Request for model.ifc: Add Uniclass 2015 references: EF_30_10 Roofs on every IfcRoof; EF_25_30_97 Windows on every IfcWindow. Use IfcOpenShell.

First a look at what the model holds.

```python
import ifcopenshell

model = ifcopenshell.open("model.ifc")
print(model.schema)
print("classifications:", [c.Name for c in model.by_type("IfcClassification")])
for ifc_class in ("IfcDoor", "IfcRoof", "IfcStair", "IfcWall", "IfcWindow"):
    print(ifc_class, len(model.by_type(ifc_class)))
```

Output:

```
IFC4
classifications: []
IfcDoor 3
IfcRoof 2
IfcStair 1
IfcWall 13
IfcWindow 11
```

```python
import ifcopenshell
import ifcopenshell.api.classification

model = ifcopenshell.open("model.ifc")

system = ifcopenshell.api.classification.add_classification(model, classification="Uniclass 2015")

codes = {
    "IfcRoof": ("EF_30_10", "Roofs"),
    "IfcWindow": ("EF_25_30_97", "Windows"),
}
for ifc_class, (code, name) in codes.items():
    products = model.by_type(ifc_class)
    ifcopenshell.api.classification.add_reference(
        model, products=products, classification=system, identification=code, name=name
    )
    print(code, len(products))

model.write("model_rev.ifc")
```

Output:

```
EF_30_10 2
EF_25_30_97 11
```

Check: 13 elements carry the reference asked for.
